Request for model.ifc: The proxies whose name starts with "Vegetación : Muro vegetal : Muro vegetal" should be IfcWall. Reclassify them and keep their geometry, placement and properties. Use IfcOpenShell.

First a look at what the model holds.

```python
import re

import ifcopenshell

model = ifcopenshell.open("model.ifc")
print(model.schema)
seen = {}
for e in model.by_type("IfcBuildingElementProxy"):
    name = re.sub(r":\d+(:\d+)?$", "", e.Name or "")  # drop the element id that some exporters append
    seen[name] = seen.get(name, 0) + 1
for name, count in sorted(seen.items()):
    print(count, "x", name)
```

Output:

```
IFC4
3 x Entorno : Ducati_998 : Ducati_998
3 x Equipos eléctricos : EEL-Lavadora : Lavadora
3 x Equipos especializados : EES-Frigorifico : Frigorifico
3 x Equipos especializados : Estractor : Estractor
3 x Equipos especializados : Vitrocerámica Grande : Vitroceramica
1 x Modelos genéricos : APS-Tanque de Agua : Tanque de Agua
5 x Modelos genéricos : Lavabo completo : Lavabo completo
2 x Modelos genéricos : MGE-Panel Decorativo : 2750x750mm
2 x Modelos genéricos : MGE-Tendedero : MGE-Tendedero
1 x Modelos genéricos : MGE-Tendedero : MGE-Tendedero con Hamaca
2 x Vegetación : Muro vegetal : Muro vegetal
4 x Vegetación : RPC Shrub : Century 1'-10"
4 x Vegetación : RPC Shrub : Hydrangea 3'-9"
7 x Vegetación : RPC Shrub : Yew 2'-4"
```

```python
import ifcopenshell
import ifcopenshell.api.root

model = ifcopenshell.open("model.ifc")

proxies = [e.id() for e in model.by_type("IfcBuildingElementProxy") if (e.Name or "").startswith("Vegetación : Muro vegetal : Muro vegetal")]
for step_id in proxies:
    proxy = model.by_id(step_id)
    # Reclassifying a typed element also reclassifies its type and the type's other occurrences.
    if proxy.is_a("IfcBuildingElementProxy"):
        ifcopenshell.api.root.reassign_class(model, product=proxy, ifc_class="IfcWall")

print(sum(model.by_id(i).is_a("IfcWall") for i in proxies), "reclassified")

model.write("model-out.ifc")
```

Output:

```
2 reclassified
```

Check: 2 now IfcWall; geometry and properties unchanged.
